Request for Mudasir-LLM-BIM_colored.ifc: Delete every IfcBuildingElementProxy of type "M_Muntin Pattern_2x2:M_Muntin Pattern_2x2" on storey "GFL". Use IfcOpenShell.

First a look at what the model holds.

```python
import ifcopenshell
import ifcopenshell.util.element

model = ifcopenshell.open("Mudasir-LLM-BIM_colored.ifc")
print(model.schema)
storey = next(s for s in model.by_type("IfcBuildingStorey") if s.Name == "GFL")
proxies = [e for e in ifcopenshell.util.element.get_decomposition(storey) if e.is_a("IfcBuildingElementProxy")]
seen = {}
for e in proxies:
    element_type = ifcopenshell.util.element.get_type(e)
    name = element_type.Name if element_type not in (None, e) else None
    seen[name] = seen.get(name, 0) + 1
for name, count in sorted(seen.items(), key=str):
    print(count, "x", name)
```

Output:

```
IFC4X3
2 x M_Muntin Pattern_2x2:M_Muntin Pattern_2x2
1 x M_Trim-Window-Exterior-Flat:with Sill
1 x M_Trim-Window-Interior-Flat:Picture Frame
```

```python
import ifcopenshell
import ifcopenshell.api.root
import ifcopenshell.util.element

model = ifcopenshell.open("Mudasir-LLM-BIM_colored.ifc")

storey = next(s for s in model.by_type("IfcBuildingStorey") if s.Name == "GFL")
proxies = [e for e in ifcopenshell.util.element.get_decomposition(storey) if e.is_a("IfcBuildingElementProxy")]
targets = [e for e in proxies if (t := ifcopenshell.util.element.get_type(e)) not in (None, e) and t.Name == "M_Muntin Pattern_2x2:M_Muntin Pattern_2x2"]

for e in targets:
    ifcopenshell.api.root.remove_product(model, product=e)
print(len(targets), "removed")

model.write("Mudasir-LLM-BIM_colored_edited.ifc")
```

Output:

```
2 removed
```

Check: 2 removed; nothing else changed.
